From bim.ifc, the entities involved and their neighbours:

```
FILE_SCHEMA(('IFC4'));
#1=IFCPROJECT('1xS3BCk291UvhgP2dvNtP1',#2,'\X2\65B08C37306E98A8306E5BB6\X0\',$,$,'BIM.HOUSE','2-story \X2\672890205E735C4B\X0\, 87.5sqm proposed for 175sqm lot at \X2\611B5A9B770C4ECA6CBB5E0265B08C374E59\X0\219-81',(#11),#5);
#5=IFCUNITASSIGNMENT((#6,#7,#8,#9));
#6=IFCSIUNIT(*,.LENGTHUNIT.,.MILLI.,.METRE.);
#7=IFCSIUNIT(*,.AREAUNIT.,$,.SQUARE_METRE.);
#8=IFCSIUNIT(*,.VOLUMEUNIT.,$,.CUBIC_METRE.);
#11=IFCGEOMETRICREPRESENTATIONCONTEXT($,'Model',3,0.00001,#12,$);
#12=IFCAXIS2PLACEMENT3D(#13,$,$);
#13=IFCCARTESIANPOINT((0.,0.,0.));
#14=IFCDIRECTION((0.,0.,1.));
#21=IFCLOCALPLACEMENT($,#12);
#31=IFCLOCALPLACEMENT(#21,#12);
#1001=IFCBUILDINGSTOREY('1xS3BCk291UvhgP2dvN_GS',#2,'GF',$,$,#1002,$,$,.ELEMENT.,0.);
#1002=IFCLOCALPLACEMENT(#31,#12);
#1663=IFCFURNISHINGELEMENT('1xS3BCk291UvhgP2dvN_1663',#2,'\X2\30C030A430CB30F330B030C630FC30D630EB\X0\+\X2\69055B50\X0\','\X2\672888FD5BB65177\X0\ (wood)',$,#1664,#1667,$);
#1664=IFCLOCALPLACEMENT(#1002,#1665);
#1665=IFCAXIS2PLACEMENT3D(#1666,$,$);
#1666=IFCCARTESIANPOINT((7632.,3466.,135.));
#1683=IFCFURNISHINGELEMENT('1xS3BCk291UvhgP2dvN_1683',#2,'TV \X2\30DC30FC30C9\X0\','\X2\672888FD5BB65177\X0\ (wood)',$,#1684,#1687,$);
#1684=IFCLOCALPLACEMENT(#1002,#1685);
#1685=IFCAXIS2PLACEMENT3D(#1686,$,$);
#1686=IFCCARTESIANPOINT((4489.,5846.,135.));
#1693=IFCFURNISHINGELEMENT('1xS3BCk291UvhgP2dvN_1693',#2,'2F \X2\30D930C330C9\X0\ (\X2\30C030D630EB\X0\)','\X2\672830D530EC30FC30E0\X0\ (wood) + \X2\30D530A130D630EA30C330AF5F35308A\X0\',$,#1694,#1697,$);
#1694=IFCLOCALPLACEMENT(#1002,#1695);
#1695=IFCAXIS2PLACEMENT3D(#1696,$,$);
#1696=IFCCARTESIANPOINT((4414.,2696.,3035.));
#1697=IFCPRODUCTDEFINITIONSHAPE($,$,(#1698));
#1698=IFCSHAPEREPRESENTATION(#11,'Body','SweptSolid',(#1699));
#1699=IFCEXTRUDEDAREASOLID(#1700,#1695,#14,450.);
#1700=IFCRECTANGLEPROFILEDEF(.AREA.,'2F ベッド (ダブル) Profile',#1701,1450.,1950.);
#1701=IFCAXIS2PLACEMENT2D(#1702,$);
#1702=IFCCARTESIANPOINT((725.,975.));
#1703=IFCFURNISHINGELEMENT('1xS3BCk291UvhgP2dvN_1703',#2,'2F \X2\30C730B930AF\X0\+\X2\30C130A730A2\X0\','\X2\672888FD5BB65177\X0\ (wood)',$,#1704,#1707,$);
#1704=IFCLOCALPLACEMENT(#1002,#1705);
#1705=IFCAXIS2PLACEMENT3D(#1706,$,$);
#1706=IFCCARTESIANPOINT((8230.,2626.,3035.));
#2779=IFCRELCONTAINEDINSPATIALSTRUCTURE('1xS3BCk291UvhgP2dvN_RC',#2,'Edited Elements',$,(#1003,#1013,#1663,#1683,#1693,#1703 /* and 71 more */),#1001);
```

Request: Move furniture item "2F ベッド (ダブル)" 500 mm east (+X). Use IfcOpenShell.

```python
import ifcopenshell
import ifcopenshell.api.geometry
import ifcopenshell.util.placement

model = ifcopenshell.open("bim.ifc")

item = model.by_guid("1xS3BCk291UvhgP2dvN_1693")
matrix = ifcopenshell.util.placement.get_local_placement(item.ObjectPlacement)
matrix[0, 3] += 500.0
ifcopenshell.api.geometry.edit_object_placement(model, product=item, matrix=matrix, is_si=False)

print(ifcopenshell.util.placement.get_local_placement(item.ObjectPlacement).round(3) + 0.0)

model.write("bim-out.ifc")
```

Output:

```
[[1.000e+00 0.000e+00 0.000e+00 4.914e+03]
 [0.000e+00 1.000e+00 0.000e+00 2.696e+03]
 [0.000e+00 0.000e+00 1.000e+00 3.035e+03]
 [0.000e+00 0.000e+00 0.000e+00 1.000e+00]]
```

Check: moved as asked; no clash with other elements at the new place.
